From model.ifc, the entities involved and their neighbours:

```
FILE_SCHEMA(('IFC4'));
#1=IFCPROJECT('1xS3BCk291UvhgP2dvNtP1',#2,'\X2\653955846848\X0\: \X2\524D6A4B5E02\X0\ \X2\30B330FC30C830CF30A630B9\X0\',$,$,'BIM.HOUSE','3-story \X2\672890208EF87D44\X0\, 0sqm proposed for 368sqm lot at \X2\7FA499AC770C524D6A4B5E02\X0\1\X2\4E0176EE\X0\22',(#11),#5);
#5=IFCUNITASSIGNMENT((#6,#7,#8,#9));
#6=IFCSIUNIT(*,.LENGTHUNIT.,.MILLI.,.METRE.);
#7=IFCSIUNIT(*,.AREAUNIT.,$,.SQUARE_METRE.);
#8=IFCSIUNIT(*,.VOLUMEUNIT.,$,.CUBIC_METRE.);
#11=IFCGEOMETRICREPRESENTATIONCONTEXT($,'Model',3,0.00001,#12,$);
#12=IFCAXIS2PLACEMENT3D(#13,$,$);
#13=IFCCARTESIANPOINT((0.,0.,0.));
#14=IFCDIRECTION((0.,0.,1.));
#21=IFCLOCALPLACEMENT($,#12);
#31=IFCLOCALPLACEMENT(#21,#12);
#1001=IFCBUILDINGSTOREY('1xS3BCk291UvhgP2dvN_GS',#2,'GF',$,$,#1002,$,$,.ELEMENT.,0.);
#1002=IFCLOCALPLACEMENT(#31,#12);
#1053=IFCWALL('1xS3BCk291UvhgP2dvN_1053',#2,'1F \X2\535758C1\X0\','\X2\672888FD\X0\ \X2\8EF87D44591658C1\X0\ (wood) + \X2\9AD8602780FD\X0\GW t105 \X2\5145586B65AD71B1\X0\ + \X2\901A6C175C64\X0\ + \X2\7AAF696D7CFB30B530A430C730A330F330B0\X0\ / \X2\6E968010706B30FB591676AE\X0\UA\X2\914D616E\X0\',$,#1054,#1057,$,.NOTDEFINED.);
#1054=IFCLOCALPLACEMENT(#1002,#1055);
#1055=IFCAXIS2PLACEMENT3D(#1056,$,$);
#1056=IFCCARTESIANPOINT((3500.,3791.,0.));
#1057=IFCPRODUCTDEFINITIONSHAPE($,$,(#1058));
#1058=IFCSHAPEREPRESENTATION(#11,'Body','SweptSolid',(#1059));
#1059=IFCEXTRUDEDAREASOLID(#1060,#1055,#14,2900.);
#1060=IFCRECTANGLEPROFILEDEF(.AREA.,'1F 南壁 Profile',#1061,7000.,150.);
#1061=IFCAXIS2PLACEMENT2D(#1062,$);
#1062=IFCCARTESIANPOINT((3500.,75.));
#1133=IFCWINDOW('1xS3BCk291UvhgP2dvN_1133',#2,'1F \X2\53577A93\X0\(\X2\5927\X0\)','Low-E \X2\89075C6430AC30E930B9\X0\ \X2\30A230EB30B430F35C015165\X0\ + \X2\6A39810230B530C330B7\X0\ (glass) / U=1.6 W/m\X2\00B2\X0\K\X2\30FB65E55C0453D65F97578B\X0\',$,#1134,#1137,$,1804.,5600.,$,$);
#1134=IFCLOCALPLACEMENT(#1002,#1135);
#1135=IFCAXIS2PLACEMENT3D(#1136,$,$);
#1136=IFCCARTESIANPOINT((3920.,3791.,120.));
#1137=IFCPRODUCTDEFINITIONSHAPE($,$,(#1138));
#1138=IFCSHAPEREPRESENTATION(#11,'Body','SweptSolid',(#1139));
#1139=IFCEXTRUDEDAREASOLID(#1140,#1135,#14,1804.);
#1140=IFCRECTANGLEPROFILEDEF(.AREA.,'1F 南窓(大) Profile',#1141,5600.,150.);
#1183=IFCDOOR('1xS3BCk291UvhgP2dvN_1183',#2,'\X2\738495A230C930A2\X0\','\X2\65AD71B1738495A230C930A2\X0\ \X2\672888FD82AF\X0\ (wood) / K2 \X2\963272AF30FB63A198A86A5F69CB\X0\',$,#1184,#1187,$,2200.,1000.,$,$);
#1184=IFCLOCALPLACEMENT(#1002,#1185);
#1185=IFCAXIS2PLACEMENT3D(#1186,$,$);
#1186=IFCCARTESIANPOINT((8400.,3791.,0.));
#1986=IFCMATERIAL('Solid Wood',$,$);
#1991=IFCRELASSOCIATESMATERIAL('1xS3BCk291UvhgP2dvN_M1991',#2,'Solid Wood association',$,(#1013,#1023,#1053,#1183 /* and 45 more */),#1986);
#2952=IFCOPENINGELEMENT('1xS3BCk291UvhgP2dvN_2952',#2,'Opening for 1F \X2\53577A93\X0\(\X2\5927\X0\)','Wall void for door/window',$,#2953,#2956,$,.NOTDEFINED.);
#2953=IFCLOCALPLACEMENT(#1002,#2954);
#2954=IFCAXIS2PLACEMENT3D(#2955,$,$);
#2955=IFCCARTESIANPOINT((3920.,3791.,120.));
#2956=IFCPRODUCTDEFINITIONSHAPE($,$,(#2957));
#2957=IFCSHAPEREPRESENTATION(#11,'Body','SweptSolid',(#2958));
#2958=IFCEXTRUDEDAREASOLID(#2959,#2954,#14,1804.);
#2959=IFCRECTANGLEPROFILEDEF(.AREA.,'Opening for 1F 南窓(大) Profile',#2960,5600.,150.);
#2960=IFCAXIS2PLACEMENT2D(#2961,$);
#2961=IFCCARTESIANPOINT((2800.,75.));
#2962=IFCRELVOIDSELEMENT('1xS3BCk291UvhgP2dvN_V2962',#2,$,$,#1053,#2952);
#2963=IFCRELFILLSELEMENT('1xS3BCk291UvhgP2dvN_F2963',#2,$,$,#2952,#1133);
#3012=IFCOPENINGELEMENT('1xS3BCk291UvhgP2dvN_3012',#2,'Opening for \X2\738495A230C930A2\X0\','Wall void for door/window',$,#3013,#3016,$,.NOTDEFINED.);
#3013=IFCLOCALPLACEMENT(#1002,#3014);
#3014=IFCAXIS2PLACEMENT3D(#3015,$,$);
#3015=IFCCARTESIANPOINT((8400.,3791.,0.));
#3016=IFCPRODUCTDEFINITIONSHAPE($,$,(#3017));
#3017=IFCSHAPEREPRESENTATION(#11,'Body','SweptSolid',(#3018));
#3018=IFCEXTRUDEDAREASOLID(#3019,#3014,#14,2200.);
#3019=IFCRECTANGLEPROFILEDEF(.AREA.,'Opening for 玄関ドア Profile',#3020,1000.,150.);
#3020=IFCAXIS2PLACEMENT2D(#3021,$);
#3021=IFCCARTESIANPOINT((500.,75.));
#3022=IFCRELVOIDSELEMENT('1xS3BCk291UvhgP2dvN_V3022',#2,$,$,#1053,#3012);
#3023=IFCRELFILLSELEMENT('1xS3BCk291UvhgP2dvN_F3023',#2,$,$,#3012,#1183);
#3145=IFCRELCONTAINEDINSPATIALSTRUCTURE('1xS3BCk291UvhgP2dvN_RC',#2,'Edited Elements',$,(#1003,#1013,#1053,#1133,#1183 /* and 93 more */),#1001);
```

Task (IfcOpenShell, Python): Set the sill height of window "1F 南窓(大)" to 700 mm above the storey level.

```python
import numpy as np
import ifcopenshell
import ifcopenshell.api.geometry
import ifcopenshell.geom
import ifcopenshell.util.element
import ifcopenshell.util.placement
import ifcopenshell.util.shape
import ifcopenshell.util.unit

model = ifcopenshell.open("model.ifc")
unit_scale = ifcopenshell.util.unit.calculate_unit_scale(model)

window = model.by_guid("1xS3BCk291UvhgP2dvN_1133")
opening = window.FillsVoids[0].RelatingOpeningElement
storey = ifcopenshell.util.element.get_container(window, ifc_class="IfcBuildingStorey")
level = ifcopenshell.util.placement.get_local_placement(storey.ObjectPlacement)[2, 3]

# The opening's origin need not be at the sill, so measure its lowest point.
shape = ifcopenshell.geom.create_shape(ifcopenshell.geom.settings(), opening)
bottom = ifcopenshell.util.shape.get_shape_bottom_elevation(shape, shape.geometry) / unit_scale
dz = level + 700.0 - bottom

shift = np.array([0.0, 0.0, dz])
# The window is not placed relative to its opening, so move both.
for product in (opening, window):
    matrix = ifcopenshell.util.placement.get_local_placement(product.ObjectPlacement)
    matrix[:3, 3] += shift
    ifcopenshell.api.geometry.edit_object_placement(model, product=product, matrix=matrix, is_si=False)

print(f"moved by {dz * unit_scale:+.3f} m")

model.write("model_rev.ifc")
```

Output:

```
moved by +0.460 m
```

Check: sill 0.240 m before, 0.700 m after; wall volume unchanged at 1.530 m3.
